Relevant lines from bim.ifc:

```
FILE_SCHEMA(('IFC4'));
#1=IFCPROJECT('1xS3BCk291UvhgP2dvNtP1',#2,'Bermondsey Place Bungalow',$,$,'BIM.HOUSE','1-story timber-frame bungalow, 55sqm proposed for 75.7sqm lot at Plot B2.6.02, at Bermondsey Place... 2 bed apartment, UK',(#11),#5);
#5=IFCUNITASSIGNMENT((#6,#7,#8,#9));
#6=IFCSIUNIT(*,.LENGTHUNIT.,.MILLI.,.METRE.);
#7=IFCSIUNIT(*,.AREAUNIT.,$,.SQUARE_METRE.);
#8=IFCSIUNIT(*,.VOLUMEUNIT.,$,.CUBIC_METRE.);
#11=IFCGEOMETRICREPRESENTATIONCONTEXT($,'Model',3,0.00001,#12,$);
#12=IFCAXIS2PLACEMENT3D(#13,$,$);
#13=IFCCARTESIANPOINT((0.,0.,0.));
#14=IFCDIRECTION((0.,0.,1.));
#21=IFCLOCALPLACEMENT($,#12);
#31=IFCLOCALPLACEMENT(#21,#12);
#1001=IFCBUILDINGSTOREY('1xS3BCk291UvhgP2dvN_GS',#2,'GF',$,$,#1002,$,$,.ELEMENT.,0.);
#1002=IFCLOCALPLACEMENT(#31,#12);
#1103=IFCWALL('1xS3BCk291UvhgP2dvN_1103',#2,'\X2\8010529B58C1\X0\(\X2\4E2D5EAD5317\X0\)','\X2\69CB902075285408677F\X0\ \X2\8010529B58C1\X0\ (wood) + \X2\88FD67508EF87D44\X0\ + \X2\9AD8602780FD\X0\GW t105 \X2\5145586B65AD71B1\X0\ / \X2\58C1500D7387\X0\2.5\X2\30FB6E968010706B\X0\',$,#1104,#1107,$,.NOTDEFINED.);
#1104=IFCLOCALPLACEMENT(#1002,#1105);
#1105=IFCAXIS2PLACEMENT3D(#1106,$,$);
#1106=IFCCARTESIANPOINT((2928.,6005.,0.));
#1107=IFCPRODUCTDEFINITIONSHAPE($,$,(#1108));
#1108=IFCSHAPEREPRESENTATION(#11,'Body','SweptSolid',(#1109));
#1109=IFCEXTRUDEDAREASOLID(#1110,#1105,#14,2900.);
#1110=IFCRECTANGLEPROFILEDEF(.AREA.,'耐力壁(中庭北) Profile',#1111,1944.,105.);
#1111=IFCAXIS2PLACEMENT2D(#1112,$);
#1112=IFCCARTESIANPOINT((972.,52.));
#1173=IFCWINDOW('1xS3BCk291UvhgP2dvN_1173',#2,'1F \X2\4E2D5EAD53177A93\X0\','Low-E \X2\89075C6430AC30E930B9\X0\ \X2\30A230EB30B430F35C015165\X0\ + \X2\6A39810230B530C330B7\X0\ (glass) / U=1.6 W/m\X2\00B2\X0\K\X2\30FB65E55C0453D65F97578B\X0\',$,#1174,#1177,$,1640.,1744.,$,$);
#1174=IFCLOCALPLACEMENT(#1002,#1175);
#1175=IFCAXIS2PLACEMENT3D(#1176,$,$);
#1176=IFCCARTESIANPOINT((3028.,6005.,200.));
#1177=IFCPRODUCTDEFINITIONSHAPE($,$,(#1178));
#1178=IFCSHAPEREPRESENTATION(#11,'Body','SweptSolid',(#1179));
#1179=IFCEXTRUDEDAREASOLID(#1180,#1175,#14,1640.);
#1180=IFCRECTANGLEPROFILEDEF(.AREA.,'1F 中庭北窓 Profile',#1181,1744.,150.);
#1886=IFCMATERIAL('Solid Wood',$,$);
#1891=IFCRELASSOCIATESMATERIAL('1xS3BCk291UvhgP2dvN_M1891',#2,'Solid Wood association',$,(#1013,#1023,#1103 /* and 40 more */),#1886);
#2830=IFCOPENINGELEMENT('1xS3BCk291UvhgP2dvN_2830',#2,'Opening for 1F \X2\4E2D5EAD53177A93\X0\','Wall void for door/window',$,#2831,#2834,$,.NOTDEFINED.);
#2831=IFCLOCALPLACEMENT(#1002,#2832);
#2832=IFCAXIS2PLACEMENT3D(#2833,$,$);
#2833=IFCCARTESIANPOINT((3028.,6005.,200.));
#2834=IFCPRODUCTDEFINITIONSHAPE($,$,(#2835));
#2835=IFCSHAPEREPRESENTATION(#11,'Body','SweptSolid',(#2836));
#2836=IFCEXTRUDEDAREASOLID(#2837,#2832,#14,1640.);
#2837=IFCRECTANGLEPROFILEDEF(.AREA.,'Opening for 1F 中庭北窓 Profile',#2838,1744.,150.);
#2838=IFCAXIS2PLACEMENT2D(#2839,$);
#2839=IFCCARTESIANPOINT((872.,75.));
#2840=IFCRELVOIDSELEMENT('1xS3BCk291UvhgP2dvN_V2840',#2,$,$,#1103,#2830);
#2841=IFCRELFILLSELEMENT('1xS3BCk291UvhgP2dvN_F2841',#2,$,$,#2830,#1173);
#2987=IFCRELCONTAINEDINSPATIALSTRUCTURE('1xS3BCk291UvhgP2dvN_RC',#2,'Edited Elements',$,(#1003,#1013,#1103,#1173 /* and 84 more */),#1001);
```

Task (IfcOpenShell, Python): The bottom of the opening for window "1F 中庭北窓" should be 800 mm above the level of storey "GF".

```python
import numpy as np
import ifcopenshell
import ifcopenshell.api.geometry
import ifcopenshell.geom
import ifcopenshell.util.element
import ifcopenshell.util.placement
import ifcopenshell.util.shape
import ifcopenshell.util.unit

model = ifcopenshell.open("bim.ifc")
unit_scale = ifcopenshell.util.unit.calculate_unit_scale(model)

window = model.by_guid("1xS3BCk291UvhgP2dvN_1173")
opening = window.FillsVoids[0].RelatingOpeningElement
storey = ifcopenshell.util.element.get_container(window, ifc_class="IfcBuildingStorey")
level = ifcopenshell.util.placement.get_local_placement(storey.ObjectPlacement)[2, 3]

# The opening's origin need not be at the sill, so measure its lowest point.
shape = ifcopenshell.geom.create_shape(ifcopenshell.geom.settings(), opening)
bottom = ifcopenshell.util.shape.get_shape_bottom_elevation(shape, shape.geometry) / unit_scale
dz = level + 800.0 - bottom

shift = np.array([0.0, 0.0, dz])
# The window is not placed relative to its opening, so move both.
for product in (opening, window):
    matrix = ifcopenshell.util.placement.get_local_placement(product.ObjectPlacement)
    matrix[:3, 3] += shift
    ifcopenshell.api.geometry.edit_object_placement(model, product=product, matrix=matrix, is_si=False)

print(f"moved by {dz * unit_scale:+.3f} m")

model.write("bim-out.ifc")
```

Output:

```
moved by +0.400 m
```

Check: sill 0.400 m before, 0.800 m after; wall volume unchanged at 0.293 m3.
